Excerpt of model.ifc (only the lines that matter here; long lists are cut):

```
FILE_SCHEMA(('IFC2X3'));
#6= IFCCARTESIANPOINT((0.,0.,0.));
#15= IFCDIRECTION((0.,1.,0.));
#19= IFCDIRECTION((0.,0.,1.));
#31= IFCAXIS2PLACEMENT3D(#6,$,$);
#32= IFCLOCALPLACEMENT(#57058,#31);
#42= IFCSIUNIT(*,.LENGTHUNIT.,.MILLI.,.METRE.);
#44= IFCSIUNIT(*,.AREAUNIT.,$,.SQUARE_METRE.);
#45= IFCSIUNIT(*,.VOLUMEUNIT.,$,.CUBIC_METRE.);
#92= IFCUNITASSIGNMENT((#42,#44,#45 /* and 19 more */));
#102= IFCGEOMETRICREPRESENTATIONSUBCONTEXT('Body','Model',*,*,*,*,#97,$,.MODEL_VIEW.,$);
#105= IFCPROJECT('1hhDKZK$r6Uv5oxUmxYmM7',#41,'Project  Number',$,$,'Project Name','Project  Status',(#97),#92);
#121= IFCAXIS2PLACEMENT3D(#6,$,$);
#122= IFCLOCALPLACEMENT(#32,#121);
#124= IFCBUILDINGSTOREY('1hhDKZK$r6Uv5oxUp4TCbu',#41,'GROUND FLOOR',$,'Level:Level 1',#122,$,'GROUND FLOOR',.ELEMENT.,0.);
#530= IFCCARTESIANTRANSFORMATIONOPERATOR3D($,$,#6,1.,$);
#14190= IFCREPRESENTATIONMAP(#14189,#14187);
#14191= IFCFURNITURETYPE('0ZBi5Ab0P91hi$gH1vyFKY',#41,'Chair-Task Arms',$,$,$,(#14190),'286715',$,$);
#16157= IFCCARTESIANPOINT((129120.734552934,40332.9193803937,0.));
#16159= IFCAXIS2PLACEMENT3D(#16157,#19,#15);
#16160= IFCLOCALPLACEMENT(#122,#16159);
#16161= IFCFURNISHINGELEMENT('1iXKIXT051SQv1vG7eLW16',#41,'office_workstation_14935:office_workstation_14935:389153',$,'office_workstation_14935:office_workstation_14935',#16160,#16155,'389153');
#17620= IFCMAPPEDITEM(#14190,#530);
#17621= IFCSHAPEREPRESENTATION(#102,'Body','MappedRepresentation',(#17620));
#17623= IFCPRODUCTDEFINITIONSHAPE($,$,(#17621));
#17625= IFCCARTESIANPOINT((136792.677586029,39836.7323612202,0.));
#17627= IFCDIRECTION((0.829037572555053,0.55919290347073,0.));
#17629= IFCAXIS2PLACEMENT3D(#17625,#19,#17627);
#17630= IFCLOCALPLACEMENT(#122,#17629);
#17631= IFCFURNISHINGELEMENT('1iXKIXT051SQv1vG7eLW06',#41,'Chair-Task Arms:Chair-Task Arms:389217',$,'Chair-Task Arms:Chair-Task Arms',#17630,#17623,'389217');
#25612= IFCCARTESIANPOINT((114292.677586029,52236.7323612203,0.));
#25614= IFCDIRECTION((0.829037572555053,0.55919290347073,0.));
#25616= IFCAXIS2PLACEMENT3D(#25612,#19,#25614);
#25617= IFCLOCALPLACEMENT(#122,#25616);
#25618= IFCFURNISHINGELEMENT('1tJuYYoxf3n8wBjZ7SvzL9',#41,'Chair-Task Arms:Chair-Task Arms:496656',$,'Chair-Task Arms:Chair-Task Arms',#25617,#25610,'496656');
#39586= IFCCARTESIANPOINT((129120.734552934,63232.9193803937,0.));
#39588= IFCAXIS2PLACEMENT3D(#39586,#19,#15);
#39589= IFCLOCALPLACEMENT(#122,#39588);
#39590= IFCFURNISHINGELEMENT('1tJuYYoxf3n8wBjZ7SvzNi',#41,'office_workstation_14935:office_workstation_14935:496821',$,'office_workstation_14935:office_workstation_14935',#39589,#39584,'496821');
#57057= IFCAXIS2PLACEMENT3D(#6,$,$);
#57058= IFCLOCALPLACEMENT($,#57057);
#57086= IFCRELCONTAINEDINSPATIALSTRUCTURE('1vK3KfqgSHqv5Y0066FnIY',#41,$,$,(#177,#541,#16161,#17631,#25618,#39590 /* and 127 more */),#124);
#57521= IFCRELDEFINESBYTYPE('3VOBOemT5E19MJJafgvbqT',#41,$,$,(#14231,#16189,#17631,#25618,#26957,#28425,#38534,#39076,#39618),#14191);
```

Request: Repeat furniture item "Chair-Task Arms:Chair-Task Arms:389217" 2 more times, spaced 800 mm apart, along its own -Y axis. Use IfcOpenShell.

```python
import ifcopenshell
import ifcopenshell.api.geometry
import ifcopenshell.api.root
import ifcopenshell.util.element
import ifcopenshell.util.placement
import ifcopenshell.util.unit

model = ifcopenshell.open("model.ifc")
unit_scale = ifcopenshell.util.unit.calculate_unit_scale(model)


def reuse_history(source, copy):
    """copy_class also copies each property set's owner history, people and application; keep the originals."""
    for rel in copy.IsDefinedBy:
        if rel.is_a("IfcRelDefinesByProperties") and (history := rel.RelatingPropertyDefinition.OwnerHistory):
            rel.RelatingPropertyDefinition.OwnerHistory = source.OwnerHistory
            ifcopenshell.util.element.remove_deep2(model, history)


source = model.by_guid("1iXKIXT051SQv1vG7eLW06")
base = ifcopenshell.util.placement.get_local_placement(source.ObjectPlacement)
step = -base[:3, 1] * 0.8 / unit_scale

for i in range(1, 3):
    copy = ifcopenshell.api.root.copy_class(model, product=source)
    copy.Representation = ifcopenshell.util.element.copy_deep(
        model, source.Representation, exclude=["IfcGeometricRepresentationContext", "IfcRepresentationMap"]
    )
    copy.Name = "Chair-Task Arms:Chair-Task Arms"
    copy.Tag = None
    reuse_history(source, copy)
    matrix = base.copy()
    matrix[:3, 3] += i * step
    print("added at", matrix[:3, 3].round(3) + 0.0)
    ifcopenshell.api.geometry.edit_object_placement(model, product=copy, matrix=matrix, is_si=False)

model.write("model_edited.ifc")
```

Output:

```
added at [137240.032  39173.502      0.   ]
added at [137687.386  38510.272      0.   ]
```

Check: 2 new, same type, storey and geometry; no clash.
